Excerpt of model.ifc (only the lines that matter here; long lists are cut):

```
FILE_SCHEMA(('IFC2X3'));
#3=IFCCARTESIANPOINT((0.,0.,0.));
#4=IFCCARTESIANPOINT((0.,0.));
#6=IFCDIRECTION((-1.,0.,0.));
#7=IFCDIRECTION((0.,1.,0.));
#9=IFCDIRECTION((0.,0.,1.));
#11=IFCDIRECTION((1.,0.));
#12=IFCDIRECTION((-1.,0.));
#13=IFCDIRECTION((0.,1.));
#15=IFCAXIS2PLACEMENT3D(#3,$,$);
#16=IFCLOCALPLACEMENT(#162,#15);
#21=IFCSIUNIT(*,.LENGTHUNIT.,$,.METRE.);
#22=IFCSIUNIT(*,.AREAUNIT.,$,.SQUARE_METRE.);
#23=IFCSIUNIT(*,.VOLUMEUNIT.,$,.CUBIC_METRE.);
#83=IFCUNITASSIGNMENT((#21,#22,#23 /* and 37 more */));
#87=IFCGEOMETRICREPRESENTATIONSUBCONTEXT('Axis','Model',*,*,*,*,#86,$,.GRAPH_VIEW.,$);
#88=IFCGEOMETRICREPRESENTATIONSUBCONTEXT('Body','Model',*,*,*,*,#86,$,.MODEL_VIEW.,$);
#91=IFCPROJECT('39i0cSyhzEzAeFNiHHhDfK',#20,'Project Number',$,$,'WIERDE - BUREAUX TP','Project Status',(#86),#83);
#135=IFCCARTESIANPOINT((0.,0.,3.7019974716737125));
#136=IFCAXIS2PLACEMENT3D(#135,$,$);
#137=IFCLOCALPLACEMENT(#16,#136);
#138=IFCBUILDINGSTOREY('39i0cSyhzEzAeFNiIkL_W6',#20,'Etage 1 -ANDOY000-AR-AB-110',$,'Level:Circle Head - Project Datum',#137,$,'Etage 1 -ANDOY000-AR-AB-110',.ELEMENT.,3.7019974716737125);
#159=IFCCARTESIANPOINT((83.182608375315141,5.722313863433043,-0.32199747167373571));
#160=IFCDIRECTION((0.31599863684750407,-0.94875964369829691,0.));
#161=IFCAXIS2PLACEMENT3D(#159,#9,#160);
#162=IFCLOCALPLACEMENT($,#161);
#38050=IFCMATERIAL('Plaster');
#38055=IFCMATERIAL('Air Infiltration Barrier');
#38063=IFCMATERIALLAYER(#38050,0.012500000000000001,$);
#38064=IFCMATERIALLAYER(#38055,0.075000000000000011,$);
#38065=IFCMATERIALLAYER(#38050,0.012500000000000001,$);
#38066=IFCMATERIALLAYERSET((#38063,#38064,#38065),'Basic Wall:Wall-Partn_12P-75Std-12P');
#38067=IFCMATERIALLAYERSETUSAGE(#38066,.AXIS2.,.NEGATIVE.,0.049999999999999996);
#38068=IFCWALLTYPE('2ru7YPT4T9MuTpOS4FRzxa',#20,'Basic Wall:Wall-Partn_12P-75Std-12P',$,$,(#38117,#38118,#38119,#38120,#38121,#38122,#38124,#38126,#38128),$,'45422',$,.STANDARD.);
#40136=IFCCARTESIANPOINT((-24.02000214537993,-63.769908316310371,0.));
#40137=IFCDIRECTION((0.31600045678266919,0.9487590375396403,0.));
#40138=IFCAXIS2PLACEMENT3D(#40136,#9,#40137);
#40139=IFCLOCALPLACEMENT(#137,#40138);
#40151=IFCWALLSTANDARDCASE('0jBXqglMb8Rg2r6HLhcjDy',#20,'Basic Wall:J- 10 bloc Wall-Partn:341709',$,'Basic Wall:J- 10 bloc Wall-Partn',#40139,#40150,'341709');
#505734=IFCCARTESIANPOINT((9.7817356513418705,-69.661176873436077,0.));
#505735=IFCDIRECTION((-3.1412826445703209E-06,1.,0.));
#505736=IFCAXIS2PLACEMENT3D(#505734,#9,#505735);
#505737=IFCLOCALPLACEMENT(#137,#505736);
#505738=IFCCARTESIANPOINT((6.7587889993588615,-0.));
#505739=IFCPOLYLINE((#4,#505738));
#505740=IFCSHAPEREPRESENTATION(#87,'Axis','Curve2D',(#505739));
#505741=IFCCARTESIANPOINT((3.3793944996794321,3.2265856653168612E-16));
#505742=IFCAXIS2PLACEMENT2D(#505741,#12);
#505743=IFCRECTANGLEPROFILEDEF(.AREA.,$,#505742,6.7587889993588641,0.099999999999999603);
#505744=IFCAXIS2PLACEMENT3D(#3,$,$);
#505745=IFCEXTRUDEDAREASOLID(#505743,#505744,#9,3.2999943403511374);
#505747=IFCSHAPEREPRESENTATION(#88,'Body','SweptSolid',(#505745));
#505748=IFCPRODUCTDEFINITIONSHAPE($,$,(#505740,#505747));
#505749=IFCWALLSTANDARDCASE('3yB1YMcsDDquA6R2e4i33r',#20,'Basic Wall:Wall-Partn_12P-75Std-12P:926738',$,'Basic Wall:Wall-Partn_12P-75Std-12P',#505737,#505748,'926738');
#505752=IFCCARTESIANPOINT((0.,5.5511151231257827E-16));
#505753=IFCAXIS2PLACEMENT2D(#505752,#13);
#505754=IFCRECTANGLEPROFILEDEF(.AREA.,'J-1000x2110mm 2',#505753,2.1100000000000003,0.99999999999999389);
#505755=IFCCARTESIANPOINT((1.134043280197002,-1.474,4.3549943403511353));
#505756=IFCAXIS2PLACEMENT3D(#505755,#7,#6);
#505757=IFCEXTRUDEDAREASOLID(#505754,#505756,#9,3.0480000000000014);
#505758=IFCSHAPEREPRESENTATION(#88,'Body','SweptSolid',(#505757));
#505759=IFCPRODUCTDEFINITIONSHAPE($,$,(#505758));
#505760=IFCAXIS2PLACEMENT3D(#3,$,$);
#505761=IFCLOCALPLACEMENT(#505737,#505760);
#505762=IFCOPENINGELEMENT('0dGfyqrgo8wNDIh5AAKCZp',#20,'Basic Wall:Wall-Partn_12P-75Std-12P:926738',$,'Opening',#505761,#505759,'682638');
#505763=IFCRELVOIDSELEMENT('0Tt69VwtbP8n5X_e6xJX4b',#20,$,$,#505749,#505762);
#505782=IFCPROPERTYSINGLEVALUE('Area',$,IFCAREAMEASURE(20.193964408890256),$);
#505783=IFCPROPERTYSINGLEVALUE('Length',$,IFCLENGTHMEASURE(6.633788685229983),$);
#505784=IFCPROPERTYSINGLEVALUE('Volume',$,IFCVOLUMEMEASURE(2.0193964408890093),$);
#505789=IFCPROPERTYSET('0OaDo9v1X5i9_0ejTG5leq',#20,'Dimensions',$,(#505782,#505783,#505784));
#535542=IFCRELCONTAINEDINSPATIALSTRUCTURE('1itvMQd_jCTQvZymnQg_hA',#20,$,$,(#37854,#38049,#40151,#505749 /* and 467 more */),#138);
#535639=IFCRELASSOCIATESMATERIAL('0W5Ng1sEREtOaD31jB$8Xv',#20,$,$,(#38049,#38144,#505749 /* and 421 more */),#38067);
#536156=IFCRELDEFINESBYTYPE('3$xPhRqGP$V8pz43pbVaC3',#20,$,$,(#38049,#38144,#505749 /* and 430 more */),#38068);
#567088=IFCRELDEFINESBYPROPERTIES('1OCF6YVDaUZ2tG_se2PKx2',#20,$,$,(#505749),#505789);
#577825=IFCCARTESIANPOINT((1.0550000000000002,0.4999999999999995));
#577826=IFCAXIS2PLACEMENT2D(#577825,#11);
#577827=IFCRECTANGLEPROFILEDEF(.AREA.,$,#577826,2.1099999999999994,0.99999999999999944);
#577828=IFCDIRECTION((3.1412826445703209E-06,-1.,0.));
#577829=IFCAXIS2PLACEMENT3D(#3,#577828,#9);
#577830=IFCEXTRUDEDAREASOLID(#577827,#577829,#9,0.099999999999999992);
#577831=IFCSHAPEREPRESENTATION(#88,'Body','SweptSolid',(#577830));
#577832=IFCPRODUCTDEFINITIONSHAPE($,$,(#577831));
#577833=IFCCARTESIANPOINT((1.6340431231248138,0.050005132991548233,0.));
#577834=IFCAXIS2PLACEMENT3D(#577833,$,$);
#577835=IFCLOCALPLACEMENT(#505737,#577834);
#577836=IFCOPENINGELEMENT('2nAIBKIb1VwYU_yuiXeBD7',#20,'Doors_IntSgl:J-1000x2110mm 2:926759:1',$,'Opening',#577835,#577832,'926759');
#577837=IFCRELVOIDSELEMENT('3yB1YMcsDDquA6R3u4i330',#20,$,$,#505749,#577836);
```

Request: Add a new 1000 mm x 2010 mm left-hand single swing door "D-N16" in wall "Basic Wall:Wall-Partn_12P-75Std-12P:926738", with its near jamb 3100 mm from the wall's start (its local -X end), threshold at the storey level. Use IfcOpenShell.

```python
import numpy as np
import ifcopenshell
import ifcopenshell.api.feature
import ifcopenshell.api.geometry
import ifcopenshell.api.pset
import ifcopenshell.api.root
import ifcopenshell.api.spatial
import ifcopenshell.api.type
import ifcopenshell.geom
import ifcopenshell.util.element
import ifcopenshell.util.placement
import ifcopenshell.util.representation
import ifcopenshell.util.shape
import ifcopenshell.util.unit

model = ifcopenshell.open("model.ifc")
unit_scale = ifcopenshell.util.unit.calculate_unit_scale(model)
area_scale = ifcopenshell.util.unit.calculate_unit_scale(model, "AREAUNIT")
volume_scale = ifcopenshell.util.unit.calculate_unit_scale(model, "VOLUMEUNIT")
settings = ifcopenshell.geom.settings()


def volume(element):
    """Net volume in cubic metres, openings subtracted."""
    shape = ifcopenshell.geom.create_shape(settings, element)
    return ifcopenshell.util.shape.get_volume(shape.geometry)


wall = model.by_id(505749)
storey = ifcopenshell.util.element.get_container(wall, ifc_class="IfcBuildingStorey")
context = ifcopenshell.util.representation.get_context(model, "Model", "Body", "MODEL_VIEW")
before = volume(wall)

width, height, from_end, sill = 1, 2.01, 3.1, 0.0  # metres

# The wall runs along its own X axis, and the end named is its -X end.
wall_shape = ifcopenshell.geom.create_shape(settings, wall)
x, y, z = ifcopenshell.util.shape.get_vertices(wall_shape.geometry).T
start = x.min() + from_end
face, thickness = float(y.min()), float(y.max() - y.min())
wall_matrix = ifcopenshell.util.placement.get_local_placement(wall.ObjectPlacement)
level = ifcopenshell.util.placement.get_local_placement(storey.ObjectPlacement)[2, 3]


def in_wall(x, y):
    """Placement at x, y metres in the wall's axes, at sill height."""
    matrix = wall_matrix.copy()
    matrix[:, 3] = wall_matrix @ np.array([x / unit_scale, y / unit_scale, 0.0, 1.0])
    matrix[2, 3] = level + sill / unit_scale
    return matrix


# Opening: a box that overshoots both wall faces by 50 mm.
opening = ifcopenshell.api.root.create_entity(model, ifc_class="IfcOpeningElement")
box = ifcopenshell.api.geometry.add_wall_representation(
    model, context=context, length=width, height=height, thickness=thickness + 0.1
)
ifcopenshell.api.geometry.assign_representation(model, product=opening, representation=box)
ifcopenshell.api.geometry.edit_object_placement(model, product=opening, matrix=in_wall(start, face - 0.05), is_si=False)
ifcopenshell.api.feature.add_feature(model, feature=opening, element=wall)

door = ifcopenshell.api.root.create_entity(model, ifc_class="IfcDoor", name="D-N16")
door.OverallWidth, door.OverallHeight = width / unit_scale, height / unit_scale
body = ifcopenshell.api.geometry.add_door_representation(
    model,
    context=context,
    overall_width=door.OverallWidth,
    overall_height=door.OverallHeight,
    operation_type="SINGLE_SWING_LEFT",
    lining_properties={"LiningDepth": thickness / unit_scale, "ThresholdDepth": thickness / unit_scale},
)
ifcopenshell.api.geometry.assign_representation(model, product=door, representation=body)
ifcopenshell.api.spatial.assign_container(model, products=[door], relating_structure=storey)
fills = ifcopenshell.api.feature.add_filling(model, opening=opening, element=door)
fills.OwnerHistory = door.OwnerHistory  # required in IFC2X3

# IFC2X3 keeps the operation on the door style.
style = ifcopenshell.api.root.create_entity(model, ifc_class="IfcDoorStyle", name="D-N16")
style.OperationType, style.ConstructionType = "SINGLE_SWING_LEFT", "NOTDEFINED"
style.ParameterTakesPrecedence = style.Sizeable = False
ifcopenshell.api.type.assign_type(model, related_objects=[door], relating_type=style)

# The lining spans the wall, so the door starts at the wall face.
ifcopenshell.api.geometry.edit_object_placement(model, product=door, matrix=in_wall(start, face), is_si=False)

after = volume(wall)

# Update the wall's stored quantities.
pset = model.by_id(ifcopenshell.util.element.get_pset(wall, "Dimensions", should_inherit=False)["id"])
ifcopenshell.api.pset.edit_pset(model, pset=pset, properties={
    "Area": model.create_entity("IfcAreaMeasure", after / thickness / area_scale),
    "Volume": model.create_entity("IfcVolumeMeasure", after / volume_scale),
})

print(f"wall volume {before:.3f} -> {after:.3f} m3")

model.write("model_rev.ifc")
```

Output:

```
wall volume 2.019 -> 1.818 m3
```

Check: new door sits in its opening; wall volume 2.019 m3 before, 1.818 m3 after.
